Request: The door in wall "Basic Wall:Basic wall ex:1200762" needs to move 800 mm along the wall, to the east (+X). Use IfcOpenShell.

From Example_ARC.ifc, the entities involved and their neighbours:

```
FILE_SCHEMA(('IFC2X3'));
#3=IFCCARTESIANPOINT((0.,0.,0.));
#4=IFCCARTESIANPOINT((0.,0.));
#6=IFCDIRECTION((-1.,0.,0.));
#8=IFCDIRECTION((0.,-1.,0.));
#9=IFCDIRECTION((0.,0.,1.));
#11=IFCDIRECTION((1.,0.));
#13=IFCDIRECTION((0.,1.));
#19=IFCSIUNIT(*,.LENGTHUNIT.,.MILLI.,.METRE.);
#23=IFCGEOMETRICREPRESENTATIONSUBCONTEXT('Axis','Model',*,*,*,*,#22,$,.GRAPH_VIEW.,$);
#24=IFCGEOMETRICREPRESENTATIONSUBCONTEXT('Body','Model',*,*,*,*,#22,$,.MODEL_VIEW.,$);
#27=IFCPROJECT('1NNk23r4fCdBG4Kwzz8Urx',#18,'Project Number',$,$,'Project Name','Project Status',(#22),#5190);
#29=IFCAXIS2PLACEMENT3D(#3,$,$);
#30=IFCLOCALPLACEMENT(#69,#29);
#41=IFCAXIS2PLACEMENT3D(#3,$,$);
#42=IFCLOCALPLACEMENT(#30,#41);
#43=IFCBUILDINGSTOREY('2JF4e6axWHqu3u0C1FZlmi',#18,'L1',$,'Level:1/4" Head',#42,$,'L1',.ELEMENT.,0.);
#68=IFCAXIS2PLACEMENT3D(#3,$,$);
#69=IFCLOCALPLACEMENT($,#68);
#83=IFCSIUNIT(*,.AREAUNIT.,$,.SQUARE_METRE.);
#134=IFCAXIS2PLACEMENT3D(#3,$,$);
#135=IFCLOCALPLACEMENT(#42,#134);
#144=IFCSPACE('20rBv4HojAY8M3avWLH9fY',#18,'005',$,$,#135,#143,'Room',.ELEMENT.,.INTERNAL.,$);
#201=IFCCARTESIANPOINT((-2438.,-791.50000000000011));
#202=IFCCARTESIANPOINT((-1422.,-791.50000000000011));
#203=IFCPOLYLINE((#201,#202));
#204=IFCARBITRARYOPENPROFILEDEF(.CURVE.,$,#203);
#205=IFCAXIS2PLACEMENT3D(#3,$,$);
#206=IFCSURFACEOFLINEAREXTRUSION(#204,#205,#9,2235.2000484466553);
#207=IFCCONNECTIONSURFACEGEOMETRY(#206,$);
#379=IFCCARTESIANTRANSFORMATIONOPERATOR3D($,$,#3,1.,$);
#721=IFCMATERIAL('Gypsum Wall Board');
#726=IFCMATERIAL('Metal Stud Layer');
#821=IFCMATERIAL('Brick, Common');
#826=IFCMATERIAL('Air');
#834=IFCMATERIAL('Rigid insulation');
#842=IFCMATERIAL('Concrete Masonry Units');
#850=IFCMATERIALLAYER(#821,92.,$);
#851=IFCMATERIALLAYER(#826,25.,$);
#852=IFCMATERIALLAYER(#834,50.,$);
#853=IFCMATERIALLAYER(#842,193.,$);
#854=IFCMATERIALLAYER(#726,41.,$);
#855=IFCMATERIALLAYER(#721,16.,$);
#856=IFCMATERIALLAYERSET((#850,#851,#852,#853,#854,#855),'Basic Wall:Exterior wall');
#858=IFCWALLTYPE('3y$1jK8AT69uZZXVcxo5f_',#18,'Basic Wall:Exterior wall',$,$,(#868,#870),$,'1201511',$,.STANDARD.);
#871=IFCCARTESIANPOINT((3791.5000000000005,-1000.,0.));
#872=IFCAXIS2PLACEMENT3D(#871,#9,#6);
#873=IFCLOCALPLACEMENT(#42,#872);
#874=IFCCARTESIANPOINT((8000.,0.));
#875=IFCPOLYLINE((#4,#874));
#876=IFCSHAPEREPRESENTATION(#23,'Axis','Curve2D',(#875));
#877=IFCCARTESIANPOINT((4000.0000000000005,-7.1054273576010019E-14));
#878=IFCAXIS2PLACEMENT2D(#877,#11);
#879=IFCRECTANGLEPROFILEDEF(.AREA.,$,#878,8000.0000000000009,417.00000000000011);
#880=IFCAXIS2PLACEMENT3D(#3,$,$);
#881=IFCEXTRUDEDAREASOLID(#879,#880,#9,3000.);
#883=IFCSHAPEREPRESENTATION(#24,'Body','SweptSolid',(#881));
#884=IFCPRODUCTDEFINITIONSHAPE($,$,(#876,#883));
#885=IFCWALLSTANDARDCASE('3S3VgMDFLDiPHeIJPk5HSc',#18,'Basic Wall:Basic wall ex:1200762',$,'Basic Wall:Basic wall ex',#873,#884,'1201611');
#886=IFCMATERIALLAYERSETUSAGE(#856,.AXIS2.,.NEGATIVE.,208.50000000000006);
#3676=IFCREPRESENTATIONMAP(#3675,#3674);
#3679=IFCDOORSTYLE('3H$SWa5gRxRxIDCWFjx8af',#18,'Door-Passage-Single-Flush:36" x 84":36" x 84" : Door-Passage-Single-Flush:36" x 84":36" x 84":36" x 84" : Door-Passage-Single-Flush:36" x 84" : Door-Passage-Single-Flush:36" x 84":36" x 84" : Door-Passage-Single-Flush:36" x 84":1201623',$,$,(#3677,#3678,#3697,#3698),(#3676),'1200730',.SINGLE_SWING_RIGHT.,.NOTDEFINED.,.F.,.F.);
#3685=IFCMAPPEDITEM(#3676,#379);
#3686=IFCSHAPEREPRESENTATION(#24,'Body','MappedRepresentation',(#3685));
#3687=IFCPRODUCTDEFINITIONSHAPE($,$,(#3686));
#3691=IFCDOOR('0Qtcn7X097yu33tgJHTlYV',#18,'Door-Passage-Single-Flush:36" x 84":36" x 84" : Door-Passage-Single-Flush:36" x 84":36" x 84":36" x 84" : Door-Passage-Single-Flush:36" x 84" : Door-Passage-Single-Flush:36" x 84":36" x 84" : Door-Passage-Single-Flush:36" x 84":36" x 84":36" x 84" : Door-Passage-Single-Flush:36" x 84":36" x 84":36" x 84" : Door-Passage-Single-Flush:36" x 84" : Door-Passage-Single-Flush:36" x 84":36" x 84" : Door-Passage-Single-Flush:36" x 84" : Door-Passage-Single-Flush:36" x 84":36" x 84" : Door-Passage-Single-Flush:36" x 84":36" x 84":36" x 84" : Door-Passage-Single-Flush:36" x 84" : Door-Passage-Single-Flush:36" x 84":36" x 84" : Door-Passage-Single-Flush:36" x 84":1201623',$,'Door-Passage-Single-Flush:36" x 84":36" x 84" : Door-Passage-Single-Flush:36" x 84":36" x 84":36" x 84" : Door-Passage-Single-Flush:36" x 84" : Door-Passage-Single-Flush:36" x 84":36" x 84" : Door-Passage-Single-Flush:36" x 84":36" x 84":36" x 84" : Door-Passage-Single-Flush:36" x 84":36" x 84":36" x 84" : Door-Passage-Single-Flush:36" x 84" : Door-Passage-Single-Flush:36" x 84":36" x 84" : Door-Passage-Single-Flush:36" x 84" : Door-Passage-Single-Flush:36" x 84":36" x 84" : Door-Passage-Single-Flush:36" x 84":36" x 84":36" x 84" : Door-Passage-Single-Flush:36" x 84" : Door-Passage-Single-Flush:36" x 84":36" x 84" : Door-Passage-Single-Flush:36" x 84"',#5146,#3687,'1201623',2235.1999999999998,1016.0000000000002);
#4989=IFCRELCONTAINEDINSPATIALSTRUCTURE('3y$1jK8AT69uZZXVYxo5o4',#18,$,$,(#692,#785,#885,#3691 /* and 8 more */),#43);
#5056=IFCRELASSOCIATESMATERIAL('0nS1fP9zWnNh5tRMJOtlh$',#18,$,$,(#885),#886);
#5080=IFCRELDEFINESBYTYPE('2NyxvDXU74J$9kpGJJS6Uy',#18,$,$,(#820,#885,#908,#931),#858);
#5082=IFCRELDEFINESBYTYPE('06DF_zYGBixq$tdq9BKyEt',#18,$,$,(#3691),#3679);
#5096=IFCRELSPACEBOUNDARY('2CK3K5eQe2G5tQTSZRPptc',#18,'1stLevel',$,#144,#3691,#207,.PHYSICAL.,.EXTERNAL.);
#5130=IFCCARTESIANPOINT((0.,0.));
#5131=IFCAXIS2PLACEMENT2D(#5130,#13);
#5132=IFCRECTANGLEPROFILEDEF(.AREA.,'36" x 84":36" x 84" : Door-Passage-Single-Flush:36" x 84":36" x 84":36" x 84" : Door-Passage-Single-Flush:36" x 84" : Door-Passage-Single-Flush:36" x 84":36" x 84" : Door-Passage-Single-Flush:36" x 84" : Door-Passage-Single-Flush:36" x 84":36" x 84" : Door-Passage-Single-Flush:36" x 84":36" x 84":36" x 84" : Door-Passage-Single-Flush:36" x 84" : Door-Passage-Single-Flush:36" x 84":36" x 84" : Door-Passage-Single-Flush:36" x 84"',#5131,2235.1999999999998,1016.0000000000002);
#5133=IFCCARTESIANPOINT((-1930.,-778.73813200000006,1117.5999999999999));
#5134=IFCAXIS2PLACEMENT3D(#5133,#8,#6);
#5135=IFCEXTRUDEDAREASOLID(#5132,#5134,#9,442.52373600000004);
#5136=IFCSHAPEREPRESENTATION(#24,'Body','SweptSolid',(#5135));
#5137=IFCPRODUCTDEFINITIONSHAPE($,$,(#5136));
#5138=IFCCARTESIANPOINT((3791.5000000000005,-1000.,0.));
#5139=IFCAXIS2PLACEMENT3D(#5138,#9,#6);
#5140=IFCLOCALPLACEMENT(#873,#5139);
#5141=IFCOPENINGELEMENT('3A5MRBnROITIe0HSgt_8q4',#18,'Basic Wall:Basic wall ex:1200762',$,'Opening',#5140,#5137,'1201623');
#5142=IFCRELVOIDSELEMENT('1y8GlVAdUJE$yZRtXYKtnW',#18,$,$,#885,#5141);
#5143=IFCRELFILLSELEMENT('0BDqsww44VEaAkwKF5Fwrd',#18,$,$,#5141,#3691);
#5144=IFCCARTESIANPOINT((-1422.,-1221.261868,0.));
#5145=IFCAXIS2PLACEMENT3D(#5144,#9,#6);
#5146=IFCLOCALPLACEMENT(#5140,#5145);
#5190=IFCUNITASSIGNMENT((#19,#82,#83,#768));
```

```python
import numpy as np
import ifcopenshell
import ifcopenshell.api.geometry
import ifcopenshell.util.placement
import ifcopenshell.util.unit

model = ifcopenshell.open("Example_ARC.ifc")
unit_scale = ifcopenshell.util.unit.calculate_unit_scale(model)

door = model.by_id(3691)
opening = door.FillsVoids[0].RelatingOpeningElement
wall = opening.VoidsElements[0].RelatingBuildingElement

wall_matrix = ifcopenshell.util.placement.get_local_placement(wall.ObjectPlacement)
shift = wall_matrix[:3, 0] * -0.8 / unit_scale
before = ifcopenshell.util.placement.get_local_placement(door.ObjectPlacement)[:3, 3].copy()

# The door is placed relative to its opening, so it follows when the opening moves.
matrix = ifcopenshell.util.placement.get_local_placement(opening.ObjectPlacement)
matrix[:3, 3] += shift
ifcopenshell.api.geometry.edit_object_placement(
    model, product=opening, matrix=matrix, is_si=False, should_transform_children=True
)

# Space boundary surfaces are stored in each space's coordinates; move them too.
for rel in door.ProvidesBoundaries:
    if not rel.ConnectionGeometry:
        continue
    surface = rel.ConnectionGeometry.SurfaceOnRelatingElement
    space_matrix = ifcopenshell.util.placement.get_local_placement(rel.RelatingSpace.ObjectPlacement)
    point = np.array(surface.Position.Location.Coordinates) + space_matrix[:3, :3].T @ shift
    surface.Position = model.createIfcAxis2Placement3D(
        model.createIfcCartesianPoint(point.tolist()), surface.Position.Axis, surface.Position.RefDirection
    )

after = ifcopenshell.util.placement.get_local_placement(door.ObjectPlacement)[:3, 3]
print("door moved by", (after - before).round(3) + 0.0)

model.write("Example_ARC_rev.ifc")
```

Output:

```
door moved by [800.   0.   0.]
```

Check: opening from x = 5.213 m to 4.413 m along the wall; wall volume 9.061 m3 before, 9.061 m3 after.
